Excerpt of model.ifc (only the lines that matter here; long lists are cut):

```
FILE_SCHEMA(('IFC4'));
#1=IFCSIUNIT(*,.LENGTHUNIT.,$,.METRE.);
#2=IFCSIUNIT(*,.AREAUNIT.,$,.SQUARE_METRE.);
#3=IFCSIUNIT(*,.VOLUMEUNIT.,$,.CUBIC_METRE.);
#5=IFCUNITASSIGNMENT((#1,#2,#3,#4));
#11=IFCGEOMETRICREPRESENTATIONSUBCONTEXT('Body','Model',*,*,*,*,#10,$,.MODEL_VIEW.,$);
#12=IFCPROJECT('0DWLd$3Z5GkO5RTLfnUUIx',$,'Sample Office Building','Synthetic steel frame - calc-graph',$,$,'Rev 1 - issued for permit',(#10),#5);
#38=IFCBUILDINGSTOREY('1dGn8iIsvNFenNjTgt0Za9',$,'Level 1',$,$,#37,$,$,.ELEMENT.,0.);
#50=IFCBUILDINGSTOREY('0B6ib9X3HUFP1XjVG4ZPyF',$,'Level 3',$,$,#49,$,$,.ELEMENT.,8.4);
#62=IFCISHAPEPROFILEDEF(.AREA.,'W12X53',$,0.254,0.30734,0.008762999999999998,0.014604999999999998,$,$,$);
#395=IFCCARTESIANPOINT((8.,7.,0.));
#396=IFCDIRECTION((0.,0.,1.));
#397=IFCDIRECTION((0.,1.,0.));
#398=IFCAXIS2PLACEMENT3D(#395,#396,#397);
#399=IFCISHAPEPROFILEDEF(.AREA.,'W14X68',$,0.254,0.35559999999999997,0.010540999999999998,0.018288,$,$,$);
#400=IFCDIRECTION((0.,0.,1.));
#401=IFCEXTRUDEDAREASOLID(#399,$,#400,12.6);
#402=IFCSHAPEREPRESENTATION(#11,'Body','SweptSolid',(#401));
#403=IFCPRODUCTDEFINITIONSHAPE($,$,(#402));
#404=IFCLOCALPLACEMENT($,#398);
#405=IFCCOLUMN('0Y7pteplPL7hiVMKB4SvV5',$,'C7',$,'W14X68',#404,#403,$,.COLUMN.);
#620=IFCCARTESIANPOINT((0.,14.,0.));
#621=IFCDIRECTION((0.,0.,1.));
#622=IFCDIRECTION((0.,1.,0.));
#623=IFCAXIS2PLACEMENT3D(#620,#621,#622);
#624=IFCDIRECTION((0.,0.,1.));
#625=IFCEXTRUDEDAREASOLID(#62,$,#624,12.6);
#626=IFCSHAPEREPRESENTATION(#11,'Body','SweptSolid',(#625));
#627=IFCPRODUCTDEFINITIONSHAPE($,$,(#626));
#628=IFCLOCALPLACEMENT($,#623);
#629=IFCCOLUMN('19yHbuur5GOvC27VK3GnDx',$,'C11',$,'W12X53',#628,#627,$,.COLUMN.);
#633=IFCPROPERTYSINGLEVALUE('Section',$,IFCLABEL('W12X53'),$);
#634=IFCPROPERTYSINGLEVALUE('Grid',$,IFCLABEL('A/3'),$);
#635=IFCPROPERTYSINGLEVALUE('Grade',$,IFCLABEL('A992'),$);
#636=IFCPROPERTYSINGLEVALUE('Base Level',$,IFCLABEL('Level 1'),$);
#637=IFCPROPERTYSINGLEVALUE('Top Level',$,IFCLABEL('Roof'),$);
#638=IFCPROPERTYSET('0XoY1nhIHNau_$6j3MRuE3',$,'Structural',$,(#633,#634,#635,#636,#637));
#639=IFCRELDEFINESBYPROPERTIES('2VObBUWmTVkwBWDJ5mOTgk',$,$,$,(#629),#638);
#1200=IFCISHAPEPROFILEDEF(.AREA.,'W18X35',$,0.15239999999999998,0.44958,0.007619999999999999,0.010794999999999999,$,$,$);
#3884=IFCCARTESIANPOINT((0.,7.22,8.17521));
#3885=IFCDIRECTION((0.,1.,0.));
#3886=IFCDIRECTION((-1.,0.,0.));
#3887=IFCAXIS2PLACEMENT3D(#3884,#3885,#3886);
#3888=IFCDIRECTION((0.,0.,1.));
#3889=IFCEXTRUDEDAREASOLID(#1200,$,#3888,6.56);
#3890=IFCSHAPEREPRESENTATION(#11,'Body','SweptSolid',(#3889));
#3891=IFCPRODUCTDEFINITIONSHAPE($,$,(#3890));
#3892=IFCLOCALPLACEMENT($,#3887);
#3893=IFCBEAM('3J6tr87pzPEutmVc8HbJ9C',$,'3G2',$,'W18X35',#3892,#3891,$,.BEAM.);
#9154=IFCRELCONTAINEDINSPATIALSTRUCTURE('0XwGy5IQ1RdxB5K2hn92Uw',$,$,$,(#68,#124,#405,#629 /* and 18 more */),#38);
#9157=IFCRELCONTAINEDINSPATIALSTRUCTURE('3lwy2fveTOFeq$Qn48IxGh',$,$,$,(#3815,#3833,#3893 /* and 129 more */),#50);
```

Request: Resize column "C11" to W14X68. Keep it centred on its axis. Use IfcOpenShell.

```python
import ifcopenshell
import ifcopenshell.api.pset
import ifcopenshell.util.element
import ifcopenshell.util.representation

model = ifcopenshell.open("model.ifc")

member = model.by_guid("19yHbuur5GOvC27VK3GnDx")
source = next(p for p in model.by_type("IfcIShapeProfileDef") if p.ProfileName == "W14X68")

body = ifcopenshell.util.representation.get_representation(member, "Model", "Body")
solid = body.Items[0]
old_profile = solid.SweptArea

# Copy the section's sizes but keep this member's own profile position.
profile = ifcopenshell.util.element.copy(model, source)
profile.Position = old_profile.Position
solid.SweptArea = profile
if not model.get_total_inverses(old_profile):
    ifcopenshell.util.element.remove_deep2(model, old_profile)
member.ObjectType = member.ObjectType.replace("W12X53", "W14X68")
pset = model.by_id(ifcopenshell.util.element.get_pset(member, "Structural", should_inherit=False)["id"])
ifcopenshell.api.pset.edit_pset(model, pset=pset, properties={"Section": "W14X68"})

print(solid.SweptArea)

model.write("model_updated.ifc")
```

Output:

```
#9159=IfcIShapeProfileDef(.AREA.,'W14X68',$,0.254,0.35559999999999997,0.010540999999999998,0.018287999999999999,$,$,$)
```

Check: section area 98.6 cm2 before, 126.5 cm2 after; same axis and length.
